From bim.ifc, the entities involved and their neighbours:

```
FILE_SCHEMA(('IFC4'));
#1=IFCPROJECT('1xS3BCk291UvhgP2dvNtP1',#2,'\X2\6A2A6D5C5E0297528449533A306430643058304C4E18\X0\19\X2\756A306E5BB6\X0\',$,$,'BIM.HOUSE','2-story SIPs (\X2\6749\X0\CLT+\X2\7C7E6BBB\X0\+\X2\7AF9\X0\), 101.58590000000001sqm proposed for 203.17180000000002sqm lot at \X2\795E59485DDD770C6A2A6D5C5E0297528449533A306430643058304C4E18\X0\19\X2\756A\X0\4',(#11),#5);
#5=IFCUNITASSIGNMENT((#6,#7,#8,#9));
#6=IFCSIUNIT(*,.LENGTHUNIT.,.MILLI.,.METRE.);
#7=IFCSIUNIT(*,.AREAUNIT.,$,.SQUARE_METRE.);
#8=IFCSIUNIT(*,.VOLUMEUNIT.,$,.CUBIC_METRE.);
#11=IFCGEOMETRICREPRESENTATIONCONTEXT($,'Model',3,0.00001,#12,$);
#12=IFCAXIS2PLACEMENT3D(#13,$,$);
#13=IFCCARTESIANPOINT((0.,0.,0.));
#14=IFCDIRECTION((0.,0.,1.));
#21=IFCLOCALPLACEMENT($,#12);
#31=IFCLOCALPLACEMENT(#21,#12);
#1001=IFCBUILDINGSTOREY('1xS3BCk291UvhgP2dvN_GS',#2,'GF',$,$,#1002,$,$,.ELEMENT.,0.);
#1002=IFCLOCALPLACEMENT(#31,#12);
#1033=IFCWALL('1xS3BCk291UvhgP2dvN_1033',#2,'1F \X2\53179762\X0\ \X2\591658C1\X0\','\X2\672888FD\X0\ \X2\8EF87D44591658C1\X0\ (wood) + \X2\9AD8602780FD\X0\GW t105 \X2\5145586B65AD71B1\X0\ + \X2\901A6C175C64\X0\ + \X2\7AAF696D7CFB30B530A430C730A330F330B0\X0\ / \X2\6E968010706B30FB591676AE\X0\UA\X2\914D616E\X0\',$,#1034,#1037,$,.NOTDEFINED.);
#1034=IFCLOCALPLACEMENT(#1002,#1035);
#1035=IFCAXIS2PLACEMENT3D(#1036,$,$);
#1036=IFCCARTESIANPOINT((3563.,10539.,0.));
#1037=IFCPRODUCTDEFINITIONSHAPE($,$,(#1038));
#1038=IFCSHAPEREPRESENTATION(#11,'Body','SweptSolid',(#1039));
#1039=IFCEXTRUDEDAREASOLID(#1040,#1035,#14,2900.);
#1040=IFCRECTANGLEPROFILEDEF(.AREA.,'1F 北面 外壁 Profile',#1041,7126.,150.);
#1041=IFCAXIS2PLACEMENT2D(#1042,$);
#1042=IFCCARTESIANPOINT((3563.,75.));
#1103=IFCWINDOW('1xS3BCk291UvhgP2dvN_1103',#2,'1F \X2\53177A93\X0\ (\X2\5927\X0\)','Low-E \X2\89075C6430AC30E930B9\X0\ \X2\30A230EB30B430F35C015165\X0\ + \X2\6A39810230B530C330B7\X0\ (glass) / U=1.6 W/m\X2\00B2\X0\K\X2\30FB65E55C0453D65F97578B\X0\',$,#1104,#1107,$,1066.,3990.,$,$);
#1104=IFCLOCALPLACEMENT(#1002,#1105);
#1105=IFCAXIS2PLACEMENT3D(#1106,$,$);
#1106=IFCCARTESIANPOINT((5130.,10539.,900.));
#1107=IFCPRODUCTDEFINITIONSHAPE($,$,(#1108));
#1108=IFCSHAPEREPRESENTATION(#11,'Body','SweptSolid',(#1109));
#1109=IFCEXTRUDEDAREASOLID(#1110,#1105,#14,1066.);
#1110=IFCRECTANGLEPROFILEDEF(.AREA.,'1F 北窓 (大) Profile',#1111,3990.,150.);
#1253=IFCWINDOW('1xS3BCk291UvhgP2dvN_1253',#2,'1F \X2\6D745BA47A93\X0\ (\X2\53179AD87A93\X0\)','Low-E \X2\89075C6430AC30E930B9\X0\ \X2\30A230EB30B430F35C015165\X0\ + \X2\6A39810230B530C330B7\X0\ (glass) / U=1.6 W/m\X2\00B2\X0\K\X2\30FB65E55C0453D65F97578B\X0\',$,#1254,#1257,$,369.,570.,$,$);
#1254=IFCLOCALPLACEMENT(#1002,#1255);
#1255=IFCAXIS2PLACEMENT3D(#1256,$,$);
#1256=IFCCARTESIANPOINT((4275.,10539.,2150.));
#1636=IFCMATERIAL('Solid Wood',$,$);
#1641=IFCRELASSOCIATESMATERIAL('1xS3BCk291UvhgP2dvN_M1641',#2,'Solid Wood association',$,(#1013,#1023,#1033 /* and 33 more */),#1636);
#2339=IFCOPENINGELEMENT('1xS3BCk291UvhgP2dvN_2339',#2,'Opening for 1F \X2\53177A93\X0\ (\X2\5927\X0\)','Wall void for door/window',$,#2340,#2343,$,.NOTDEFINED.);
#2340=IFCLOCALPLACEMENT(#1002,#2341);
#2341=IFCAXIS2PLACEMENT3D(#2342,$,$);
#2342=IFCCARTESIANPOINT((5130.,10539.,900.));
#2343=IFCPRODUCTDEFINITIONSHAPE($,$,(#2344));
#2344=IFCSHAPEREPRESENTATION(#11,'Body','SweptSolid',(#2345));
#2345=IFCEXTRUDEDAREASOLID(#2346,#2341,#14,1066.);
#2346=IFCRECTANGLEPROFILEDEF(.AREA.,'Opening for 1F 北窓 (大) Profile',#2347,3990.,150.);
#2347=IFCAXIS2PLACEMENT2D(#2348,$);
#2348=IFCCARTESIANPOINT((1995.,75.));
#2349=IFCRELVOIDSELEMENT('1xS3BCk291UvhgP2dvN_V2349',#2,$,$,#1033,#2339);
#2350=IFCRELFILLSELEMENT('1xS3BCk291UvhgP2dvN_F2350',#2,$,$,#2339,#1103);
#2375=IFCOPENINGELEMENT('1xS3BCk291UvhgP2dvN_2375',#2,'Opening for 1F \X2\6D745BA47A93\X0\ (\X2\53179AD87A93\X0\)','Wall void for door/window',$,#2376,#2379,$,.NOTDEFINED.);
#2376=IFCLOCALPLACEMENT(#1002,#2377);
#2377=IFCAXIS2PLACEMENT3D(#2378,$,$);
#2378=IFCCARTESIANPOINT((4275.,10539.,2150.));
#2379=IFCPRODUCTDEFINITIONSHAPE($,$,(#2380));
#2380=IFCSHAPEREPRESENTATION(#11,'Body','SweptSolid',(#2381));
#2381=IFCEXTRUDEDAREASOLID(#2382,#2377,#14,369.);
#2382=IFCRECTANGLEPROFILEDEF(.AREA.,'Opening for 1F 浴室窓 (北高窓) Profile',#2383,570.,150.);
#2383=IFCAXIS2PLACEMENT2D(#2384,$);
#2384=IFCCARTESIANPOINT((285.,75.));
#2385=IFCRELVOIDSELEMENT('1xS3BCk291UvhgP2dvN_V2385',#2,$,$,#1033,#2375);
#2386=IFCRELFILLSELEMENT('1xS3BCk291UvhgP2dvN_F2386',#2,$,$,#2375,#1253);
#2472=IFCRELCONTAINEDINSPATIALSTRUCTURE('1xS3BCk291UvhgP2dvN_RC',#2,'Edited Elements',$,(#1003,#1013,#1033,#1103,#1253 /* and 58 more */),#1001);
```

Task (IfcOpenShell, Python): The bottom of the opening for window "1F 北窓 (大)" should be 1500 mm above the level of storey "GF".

```python
import numpy as np
import ifcopenshell
import ifcopenshell.api.geometry
import ifcopenshell.geom
import ifcopenshell.util.element
import ifcopenshell.util.placement
import ifcopenshell.util.shape
import ifcopenshell.util.unit

model = ifcopenshell.open("bim.ifc")
unit_scale = ifcopenshell.util.unit.calculate_unit_scale(model)

window = model.by_guid("1xS3BCk291UvhgP2dvN_1103")
opening = window.FillsVoids[0].RelatingOpeningElement
storey = ifcopenshell.util.element.get_container(window, ifc_class="IfcBuildingStorey")
level = ifcopenshell.util.placement.get_local_placement(storey.ObjectPlacement)[2, 3]

# The opening's origin need not be at the sill, so measure its lowest point.
shape = ifcopenshell.geom.create_shape(ifcopenshell.geom.settings(), opening)
bottom = ifcopenshell.util.shape.get_shape_bottom_elevation(shape, shape.geometry) / unit_scale
dz = level + 1.5 / unit_scale - bottom

shift = np.array([0.0, 0.0, dz])
# The window is not placed relative to its opening, so move both.
for product in (opening, window):
    matrix = ifcopenshell.util.placement.get_local_placement(product.ObjectPlacement)
    matrix[:3, 3] += shift
    ifcopenshell.api.geometry.edit_object_placement(model, product=product, matrix=matrix, is_si=False)

print(f"moved by {dz * unit_scale:+.3f} m")

model.write("bim_updated.ifc")
```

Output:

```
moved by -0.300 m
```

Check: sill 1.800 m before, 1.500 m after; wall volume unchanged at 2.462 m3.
